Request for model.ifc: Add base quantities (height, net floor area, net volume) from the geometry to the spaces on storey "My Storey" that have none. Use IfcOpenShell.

First a look at what the model holds.

```python
import ifcopenshell
import ifcopenshell.util.element
import ifcopenshell.util.unit

model = ifcopenshell.open("model.ifc")
print(model.schema)
for unit_type in ("LENGTHUNIT", "AREAUNIT", "VOLUMEUNIT"):
    print(unit_type, ifcopenshell.util.unit.calculate_unit_scale(model, unit_type))
storey = next(s for s in model.by_type("IfcBuildingStorey") if s.Name == "My Storey")
spaces = [e for e in ifcopenshell.util.element.get_decomposition(storey) if e.is_a("IfcSpace")]
for e in sorted(spaces, key=lambda e: e.id()):
    print(e.id(), e.is_a(), e.Name, list(ifcopenshell.util.element.get_psets(e, qtos_only=True)), sep=" | ")
```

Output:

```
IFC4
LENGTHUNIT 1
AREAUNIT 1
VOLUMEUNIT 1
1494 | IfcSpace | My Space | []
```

```python
import ifcopenshell
import ifcopenshell.api.pset
import ifcopenshell.geom
import ifcopenshell.util.element
import ifcopenshell.util.shape
import ifcopenshell.util.unit

model = ifcopenshell.open("model.ifc")
unit_scale = ifcopenshell.util.unit.calculate_unit_scale(model)
area_scale = ifcopenshell.util.unit.calculate_unit_scale(model, "AREAUNIT")
volume_scale = ifcopenshell.util.unit.calculate_unit_scale(model, "VOLUMEUNIT")
settings = ifcopenshell.geom.settings()

storey = next(s for s in model.by_type("IfcBuildingStorey") if s.Name == "My Storey")
spaces = [e for e in ifcopenshell.util.element.get_decomposition(storey) if e.is_a("IfcSpace")]

for e in sorted(spaces, key=lambda e: e.id()):
    if ifcopenshell.util.element.get_psets(e, qtos_only=True, should_inherit=False):
        continue
    # Geometry comes back in metres, in the element's own axes.
    shape = ifcopenshell.geom.create_shape(settings, e)
    values = {
        "Height": ifcopenshell.util.shape.get_z(shape.geometry) / unit_scale,
        "NetFloorArea": ifcopenshell.util.shape.get_footprint_area(shape.geometry) / area_scale,
        "NetVolume": ifcopenshell.util.shape.get_volume(shape.geometry) / volume_scale,
    }
    qto = ifcopenshell.api.pset.add_qto(model, product=e, name="Qto_SpaceBaseQuantities")
    ifcopenshell.api.pset.edit_qto(model, qto=qto, properties=values)
    print(e.id(), {k: round(v, 3) for k, v in values.items()})

model.write("model_rev.ifc")
```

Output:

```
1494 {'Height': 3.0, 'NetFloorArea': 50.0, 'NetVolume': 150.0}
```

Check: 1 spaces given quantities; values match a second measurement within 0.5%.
